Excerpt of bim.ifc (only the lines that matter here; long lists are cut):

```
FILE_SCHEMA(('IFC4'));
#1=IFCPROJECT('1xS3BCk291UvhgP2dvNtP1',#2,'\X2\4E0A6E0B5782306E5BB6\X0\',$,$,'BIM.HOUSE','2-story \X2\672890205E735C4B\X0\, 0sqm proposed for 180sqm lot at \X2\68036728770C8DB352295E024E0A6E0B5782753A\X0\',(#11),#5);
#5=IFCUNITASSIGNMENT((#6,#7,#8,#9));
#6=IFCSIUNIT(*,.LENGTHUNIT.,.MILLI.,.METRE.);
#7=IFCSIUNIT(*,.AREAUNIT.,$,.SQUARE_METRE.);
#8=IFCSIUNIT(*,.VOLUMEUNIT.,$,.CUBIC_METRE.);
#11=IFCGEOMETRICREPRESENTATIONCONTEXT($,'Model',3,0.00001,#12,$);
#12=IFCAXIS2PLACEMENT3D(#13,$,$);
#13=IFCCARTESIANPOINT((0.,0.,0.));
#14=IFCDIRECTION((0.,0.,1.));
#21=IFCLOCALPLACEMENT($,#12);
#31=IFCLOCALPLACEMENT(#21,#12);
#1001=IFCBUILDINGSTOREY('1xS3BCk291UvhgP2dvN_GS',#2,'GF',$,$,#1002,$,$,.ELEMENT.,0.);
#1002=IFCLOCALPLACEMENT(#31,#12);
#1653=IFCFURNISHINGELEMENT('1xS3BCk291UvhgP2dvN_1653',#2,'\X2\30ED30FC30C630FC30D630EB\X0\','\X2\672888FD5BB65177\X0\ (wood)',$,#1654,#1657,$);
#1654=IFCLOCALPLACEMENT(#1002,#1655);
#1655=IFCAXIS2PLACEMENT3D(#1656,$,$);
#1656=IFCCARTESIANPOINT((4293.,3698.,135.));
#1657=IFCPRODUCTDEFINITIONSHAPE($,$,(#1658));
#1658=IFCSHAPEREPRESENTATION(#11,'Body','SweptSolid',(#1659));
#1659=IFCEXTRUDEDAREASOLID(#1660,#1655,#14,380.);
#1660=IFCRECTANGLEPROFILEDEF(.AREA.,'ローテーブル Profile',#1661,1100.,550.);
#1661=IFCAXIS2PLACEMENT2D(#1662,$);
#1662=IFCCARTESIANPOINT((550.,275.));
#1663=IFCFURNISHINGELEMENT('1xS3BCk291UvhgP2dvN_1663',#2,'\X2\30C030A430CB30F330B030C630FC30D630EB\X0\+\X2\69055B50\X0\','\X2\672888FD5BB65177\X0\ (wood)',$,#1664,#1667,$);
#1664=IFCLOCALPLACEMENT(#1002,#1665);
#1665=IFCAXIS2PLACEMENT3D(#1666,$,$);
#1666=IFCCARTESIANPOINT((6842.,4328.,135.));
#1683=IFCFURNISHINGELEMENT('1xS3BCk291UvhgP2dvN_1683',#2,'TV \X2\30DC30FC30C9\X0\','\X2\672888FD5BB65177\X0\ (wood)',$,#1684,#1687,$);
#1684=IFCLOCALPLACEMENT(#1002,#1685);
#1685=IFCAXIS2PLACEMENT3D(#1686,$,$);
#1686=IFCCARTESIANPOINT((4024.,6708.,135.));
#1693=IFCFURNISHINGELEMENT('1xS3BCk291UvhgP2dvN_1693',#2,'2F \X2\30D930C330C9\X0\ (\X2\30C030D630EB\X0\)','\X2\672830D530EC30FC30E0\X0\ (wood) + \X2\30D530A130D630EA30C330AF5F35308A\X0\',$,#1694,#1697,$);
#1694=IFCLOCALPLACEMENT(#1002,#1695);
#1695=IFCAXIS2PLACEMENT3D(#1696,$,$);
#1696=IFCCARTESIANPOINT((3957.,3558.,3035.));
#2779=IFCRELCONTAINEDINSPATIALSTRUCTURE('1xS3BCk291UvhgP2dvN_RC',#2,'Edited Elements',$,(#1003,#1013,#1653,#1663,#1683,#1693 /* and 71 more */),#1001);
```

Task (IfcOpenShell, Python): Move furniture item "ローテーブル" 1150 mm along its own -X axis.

```python
import ifcopenshell
import ifcopenshell.api.geometry
import ifcopenshell.util.placement

model = ifcopenshell.open("bim.ifc")

item = model.by_guid("1xS3BCk291UvhgP2dvN_1653")
matrix = ifcopenshell.util.placement.get_local_placement(item.ObjectPlacement)
matrix[:3, 3] -= matrix[:3, 0] * 1150.0
ifcopenshell.api.geometry.edit_object_placement(model, product=item, matrix=matrix, is_si=False)

print(ifcopenshell.util.placement.get_local_placement(item.ObjectPlacement).round(3) + 0.0)

model.write("bim_edited.ifc")
```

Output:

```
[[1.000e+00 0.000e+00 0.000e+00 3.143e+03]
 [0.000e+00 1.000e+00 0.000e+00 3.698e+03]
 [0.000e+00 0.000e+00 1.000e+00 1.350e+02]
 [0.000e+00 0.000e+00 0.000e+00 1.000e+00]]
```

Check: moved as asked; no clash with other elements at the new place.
